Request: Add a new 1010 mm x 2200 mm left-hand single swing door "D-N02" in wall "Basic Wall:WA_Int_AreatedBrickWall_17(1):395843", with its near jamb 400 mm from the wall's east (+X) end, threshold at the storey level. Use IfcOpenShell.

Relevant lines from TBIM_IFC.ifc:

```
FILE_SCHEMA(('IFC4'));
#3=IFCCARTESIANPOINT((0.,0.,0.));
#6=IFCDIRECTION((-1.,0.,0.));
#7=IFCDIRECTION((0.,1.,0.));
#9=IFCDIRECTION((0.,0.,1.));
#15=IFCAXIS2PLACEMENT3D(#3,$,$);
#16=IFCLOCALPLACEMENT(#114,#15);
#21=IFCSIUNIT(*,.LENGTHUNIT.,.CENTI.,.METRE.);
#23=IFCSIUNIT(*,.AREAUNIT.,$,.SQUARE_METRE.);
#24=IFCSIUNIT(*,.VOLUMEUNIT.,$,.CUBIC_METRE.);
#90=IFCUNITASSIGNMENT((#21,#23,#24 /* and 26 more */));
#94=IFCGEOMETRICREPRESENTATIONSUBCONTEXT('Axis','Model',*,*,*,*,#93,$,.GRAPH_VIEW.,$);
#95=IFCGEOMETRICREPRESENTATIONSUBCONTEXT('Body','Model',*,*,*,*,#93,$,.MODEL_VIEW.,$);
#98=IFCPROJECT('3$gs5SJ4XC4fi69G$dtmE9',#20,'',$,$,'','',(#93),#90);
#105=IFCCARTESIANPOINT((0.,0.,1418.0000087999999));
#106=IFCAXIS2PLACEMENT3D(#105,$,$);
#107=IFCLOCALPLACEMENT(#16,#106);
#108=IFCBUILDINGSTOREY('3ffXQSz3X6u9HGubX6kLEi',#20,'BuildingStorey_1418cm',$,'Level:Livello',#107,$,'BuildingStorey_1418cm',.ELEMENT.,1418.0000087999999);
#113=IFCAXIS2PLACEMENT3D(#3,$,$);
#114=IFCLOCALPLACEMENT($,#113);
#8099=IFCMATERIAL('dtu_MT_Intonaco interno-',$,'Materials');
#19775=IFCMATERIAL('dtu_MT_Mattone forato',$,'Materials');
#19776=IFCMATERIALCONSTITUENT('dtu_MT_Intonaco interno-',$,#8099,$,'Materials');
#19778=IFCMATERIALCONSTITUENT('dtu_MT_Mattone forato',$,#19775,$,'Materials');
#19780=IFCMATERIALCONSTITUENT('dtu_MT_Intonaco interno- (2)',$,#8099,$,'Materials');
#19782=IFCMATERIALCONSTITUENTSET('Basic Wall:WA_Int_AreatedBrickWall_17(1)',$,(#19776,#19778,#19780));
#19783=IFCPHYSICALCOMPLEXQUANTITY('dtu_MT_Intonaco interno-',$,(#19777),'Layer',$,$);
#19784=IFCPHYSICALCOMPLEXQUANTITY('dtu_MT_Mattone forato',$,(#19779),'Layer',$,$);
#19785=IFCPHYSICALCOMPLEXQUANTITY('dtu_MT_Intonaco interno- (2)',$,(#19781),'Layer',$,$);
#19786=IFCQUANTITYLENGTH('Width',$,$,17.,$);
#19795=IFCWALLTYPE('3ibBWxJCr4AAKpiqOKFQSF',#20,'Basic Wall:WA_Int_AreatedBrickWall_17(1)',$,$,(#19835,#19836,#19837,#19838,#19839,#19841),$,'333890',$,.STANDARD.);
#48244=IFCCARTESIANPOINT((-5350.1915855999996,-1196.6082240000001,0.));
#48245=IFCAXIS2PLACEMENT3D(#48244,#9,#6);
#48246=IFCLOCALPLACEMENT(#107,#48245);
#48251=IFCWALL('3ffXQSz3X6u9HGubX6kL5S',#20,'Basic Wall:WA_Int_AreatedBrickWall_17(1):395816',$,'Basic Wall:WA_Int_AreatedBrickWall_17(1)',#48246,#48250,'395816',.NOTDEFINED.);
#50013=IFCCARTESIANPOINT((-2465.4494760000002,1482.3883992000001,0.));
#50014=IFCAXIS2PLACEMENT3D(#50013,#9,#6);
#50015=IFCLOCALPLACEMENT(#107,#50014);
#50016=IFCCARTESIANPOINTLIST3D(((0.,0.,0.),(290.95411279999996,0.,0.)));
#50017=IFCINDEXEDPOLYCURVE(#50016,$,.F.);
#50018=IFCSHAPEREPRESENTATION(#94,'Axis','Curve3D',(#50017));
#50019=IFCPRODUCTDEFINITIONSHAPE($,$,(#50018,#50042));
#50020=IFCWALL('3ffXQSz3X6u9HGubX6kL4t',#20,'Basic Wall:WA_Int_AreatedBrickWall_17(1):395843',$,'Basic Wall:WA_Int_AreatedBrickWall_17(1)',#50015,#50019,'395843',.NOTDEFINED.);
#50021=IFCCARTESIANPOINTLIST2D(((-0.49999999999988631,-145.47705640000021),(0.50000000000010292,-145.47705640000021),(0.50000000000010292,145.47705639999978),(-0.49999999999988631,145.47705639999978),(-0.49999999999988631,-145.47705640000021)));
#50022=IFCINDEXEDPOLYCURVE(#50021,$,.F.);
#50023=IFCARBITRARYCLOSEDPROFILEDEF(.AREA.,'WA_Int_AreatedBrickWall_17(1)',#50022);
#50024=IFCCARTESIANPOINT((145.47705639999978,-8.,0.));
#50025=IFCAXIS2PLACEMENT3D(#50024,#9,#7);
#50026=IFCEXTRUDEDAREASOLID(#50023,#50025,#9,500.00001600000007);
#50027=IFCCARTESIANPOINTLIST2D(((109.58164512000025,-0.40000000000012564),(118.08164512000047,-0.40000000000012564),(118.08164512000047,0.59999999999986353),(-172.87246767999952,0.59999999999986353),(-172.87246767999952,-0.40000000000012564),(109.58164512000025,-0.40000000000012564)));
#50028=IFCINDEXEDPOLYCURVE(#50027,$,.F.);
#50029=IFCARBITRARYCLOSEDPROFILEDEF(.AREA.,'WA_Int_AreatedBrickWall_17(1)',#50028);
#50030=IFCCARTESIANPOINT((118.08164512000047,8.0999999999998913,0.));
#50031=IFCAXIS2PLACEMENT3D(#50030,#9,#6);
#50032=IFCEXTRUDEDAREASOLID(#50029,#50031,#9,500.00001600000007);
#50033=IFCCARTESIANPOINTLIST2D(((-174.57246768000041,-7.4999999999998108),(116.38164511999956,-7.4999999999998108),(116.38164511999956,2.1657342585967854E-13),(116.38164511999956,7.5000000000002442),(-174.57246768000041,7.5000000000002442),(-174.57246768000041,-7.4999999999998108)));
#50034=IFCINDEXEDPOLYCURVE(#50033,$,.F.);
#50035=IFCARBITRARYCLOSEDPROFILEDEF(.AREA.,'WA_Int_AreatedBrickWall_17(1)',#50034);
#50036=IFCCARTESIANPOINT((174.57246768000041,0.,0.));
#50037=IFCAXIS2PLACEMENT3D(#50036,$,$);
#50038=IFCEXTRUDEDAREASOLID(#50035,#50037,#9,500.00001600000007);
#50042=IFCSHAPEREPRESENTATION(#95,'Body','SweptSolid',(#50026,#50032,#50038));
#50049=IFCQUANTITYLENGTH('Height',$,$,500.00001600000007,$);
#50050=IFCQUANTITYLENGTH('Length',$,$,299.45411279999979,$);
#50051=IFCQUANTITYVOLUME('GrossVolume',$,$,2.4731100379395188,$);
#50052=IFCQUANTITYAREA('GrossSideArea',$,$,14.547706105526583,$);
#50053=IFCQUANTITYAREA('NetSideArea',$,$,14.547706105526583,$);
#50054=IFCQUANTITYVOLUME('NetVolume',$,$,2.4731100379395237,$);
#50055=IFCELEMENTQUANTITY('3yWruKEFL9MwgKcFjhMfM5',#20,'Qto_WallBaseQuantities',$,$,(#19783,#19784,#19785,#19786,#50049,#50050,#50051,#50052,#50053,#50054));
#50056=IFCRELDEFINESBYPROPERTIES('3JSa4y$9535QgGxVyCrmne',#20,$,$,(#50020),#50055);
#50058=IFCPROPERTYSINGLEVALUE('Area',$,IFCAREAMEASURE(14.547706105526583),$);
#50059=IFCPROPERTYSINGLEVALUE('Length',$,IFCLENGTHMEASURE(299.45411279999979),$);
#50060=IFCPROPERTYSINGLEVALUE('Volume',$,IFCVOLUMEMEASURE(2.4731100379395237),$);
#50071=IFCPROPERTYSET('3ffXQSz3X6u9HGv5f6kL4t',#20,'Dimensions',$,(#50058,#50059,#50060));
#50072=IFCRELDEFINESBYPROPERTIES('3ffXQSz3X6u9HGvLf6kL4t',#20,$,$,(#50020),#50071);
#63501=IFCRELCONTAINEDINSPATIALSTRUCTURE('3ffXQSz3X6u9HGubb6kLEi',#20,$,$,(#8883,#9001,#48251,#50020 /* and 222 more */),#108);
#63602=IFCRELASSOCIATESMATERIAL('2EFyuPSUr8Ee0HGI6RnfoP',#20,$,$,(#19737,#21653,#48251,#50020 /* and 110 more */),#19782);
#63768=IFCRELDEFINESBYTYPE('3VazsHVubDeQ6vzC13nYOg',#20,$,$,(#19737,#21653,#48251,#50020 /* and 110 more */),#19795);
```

```python
import numpy as np
import ifcopenshell
import ifcopenshell.api.feature
import ifcopenshell.api.geometry
import ifcopenshell.api.pset
import ifcopenshell.api.root
import ifcopenshell.api.spatial
import ifcopenshell.geom
import ifcopenshell.util.element
import ifcopenshell.util.placement
import ifcopenshell.util.representation
import ifcopenshell.util.shape
import ifcopenshell.util.unit

model = ifcopenshell.open("TBIM_IFC.ifc")
unit_scale = ifcopenshell.util.unit.calculate_unit_scale(model)
area_scale = ifcopenshell.util.unit.calculate_unit_scale(model, "AREAUNIT")
volume_scale = ifcopenshell.util.unit.calculate_unit_scale(model, "VOLUMEUNIT")
settings = ifcopenshell.geom.settings()


def volume(element):
    """Net volume in cubic metres, openings subtracted."""
    shape = ifcopenshell.geom.create_shape(settings, element)
    return ifcopenshell.util.shape.get_volume(shape.geometry)


wall = model.by_guid("3ffXQSz3X6u9HGubX6kL4t")
storey = ifcopenshell.util.element.get_container(wall, ifc_class="IfcBuildingStorey")
context = ifcopenshell.util.representation.get_context(model, "Model", "Body", "MODEL_VIEW")
before = volume(wall)

width, height, from_end, sill = 1.01, 2.2, 0.4, 0.0  # metres

# The wall runs along its own X axis, and the end named is its -X end.
wall_shape = ifcopenshell.geom.create_shape(settings, wall)
x, y, z = ifcopenshell.util.shape.get_vertices(wall_shape.geometry).T
start = x.min() + from_end
face, thickness = float(y.min()), float(y.max() - y.min())
wall_matrix = ifcopenshell.util.placement.get_local_placement(wall.ObjectPlacement)
level = ifcopenshell.util.placement.get_local_placement(storey.ObjectPlacement)[2, 3]


def in_wall(x, y):
    """Placement at x, y metres in the wall's axes, at sill height."""
    matrix = wall_matrix.copy()
    matrix[:, 3] = wall_matrix @ np.array([x / unit_scale, y / unit_scale, 0.0, 1.0])
    matrix[2, 3] = level + sill / unit_scale
    return matrix


# Opening: a box that overshoots both wall faces by 50 mm.
opening = ifcopenshell.api.root.create_entity(model, ifc_class="IfcOpeningElement", predefined_type="OPENING")
box = ifcopenshell.api.geometry.add_wall_representation(
    model, context=context, length=width, height=height, thickness=thickness + 0.1
)
ifcopenshell.api.geometry.assign_representation(model, product=opening, representation=box)
ifcopenshell.api.geometry.edit_object_placement(model, product=opening, matrix=in_wall(start, face - 0.05), is_si=False)
ifcopenshell.api.feature.add_feature(model, feature=opening, element=wall)

door = ifcopenshell.api.root.create_entity(model, ifc_class="IfcDoor", name="D-N02", predefined_type="DOOR")
door.OverallWidth, door.OverallHeight = width / unit_scale, height / unit_scale
door.OperationType = "SINGLE_SWING_LEFT"
body = ifcopenshell.api.geometry.add_door_representation(
    model,
    context=context,
    overall_width=door.OverallWidth,
    overall_height=door.OverallHeight,
    operation_type="SINGLE_SWING_LEFT",
    lining_properties={"LiningDepth": thickness / unit_scale, "ThresholdDepth": thickness / unit_scale},
)
ifcopenshell.api.geometry.assign_representation(model, product=door, representation=body)
ifcopenshell.api.spatial.assign_container(model, products=[door], relating_structure=storey)
ifcopenshell.api.feature.add_filling(model, opening=opening, element=door)

# The lining spans the wall, so the door starts at the wall face.
ifcopenshell.api.geometry.edit_object_placement(model, product=door, matrix=in_wall(start, face), is_si=False)

after = volume(wall)

# Update the wall's stored quantities.
qto = model.by_id(ifcopenshell.util.element.get_pset(wall, "Qto_WallBaseQuantities", should_inherit=False)["id"])
ifcopenshell.api.pset.edit_qto(model, qto=qto, properties={
    "NetSideArea": after / thickness / area_scale,
    "NetVolume": after / volume_scale,
})
pset = model.by_id(ifcopenshell.util.element.get_pset(wall, "Dimensions", should_inherit=False)["id"])
ifcopenshell.api.pset.edit_pset(model, pset=pset, properties={
    "Area": model.create_entity("IfcAreaMeasure", after / thickness / area_scale),
    "Volume": model.create_entity("IfcVolumeMeasure", after / volume_scale),
})

print(f"wall volume {before:.3f} -> {after:.3f} m3")

model.write("TBIM_IFC_rev.ifc")
```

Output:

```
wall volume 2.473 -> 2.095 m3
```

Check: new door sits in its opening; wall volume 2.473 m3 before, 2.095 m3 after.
